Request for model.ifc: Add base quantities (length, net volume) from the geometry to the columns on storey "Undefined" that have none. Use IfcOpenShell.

First a look at what the model holds.

```python
import ifcopenshell
import ifcopenshell.util.element
import ifcopenshell.util.unit

model = ifcopenshell.open("model.ifc")
print(model.schema)
for unit_type in ("LENGTHUNIT", "AREAUNIT", "VOLUMEUNIT"):
    print(unit_type, ifcopenshell.util.unit.calculate_unit_scale(model, unit_type))
storey = next(s for s in model.by_type("IfcBuildingStorey") if s.Name == "Undefined")
columns = [e for e in ifcopenshell.util.element.get_decomposition(storey) if e.is_a("IfcColumn")]
for e in sorted(columns, key=lambda e: e.id()):
    print(e.id(), e.is_a(), e.Name, list(ifcopenshell.util.element.get_psets(e, qtos_only=True)), sep=" | ")
```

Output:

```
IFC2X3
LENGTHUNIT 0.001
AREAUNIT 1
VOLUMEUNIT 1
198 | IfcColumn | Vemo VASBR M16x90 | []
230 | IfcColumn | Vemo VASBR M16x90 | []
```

```python
import ifcopenshell
import ifcopenshell.api.pset
import ifcopenshell.geom
import ifcopenshell.util.element
import ifcopenshell.util.shape
import ifcopenshell.util.unit

model = ifcopenshell.open("model.ifc")
unit_scale = ifcopenshell.util.unit.calculate_unit_scale(model)
volume_scale = ifcopenshell.util.unit.calculate_unit_scale(model, "VOLUMEUNIT")
settings = ifcopenshell.geom.settings()

storey = next(s for s in model.by_type("IfcBuildingStorey") if s.Name == "Undefined")
columns = [e for e in ifcopenshell.util.element.get_decomposition(storey) if e.is_a("IfcColumn")]

for e in sorted(columns, key=lambda e: e.id()):
    if ifcopenshell.util.element.get_psets(e, qtos_only=True, should_inherit=False):
        continue
    # Geometry comes back in metres, in the element's own axes.
    shape = ifcopenshell.geom.create_shape(settings, e)
    values = {
        "Length": ifcopenshell.util.shape.get_z(shape.geometry) / unit_scale,
        "NetVolume": ifcopenshell.util.shape.get_volume(shape.geometry) / volume_scale,
    }
    qto = ifcopenshell.api.pset.add_qto(model, product=e, name="BaseQuantities")
    ifcopenshell.api.pset.edit_qto(model, qto=qto, properties=values)
    print(e.id(), {k: round(v, 3) for k, v in values.items()})

model.write("model_v2.ifc")
```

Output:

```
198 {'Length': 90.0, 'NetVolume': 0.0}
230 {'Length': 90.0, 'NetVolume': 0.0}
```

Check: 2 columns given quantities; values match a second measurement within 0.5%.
